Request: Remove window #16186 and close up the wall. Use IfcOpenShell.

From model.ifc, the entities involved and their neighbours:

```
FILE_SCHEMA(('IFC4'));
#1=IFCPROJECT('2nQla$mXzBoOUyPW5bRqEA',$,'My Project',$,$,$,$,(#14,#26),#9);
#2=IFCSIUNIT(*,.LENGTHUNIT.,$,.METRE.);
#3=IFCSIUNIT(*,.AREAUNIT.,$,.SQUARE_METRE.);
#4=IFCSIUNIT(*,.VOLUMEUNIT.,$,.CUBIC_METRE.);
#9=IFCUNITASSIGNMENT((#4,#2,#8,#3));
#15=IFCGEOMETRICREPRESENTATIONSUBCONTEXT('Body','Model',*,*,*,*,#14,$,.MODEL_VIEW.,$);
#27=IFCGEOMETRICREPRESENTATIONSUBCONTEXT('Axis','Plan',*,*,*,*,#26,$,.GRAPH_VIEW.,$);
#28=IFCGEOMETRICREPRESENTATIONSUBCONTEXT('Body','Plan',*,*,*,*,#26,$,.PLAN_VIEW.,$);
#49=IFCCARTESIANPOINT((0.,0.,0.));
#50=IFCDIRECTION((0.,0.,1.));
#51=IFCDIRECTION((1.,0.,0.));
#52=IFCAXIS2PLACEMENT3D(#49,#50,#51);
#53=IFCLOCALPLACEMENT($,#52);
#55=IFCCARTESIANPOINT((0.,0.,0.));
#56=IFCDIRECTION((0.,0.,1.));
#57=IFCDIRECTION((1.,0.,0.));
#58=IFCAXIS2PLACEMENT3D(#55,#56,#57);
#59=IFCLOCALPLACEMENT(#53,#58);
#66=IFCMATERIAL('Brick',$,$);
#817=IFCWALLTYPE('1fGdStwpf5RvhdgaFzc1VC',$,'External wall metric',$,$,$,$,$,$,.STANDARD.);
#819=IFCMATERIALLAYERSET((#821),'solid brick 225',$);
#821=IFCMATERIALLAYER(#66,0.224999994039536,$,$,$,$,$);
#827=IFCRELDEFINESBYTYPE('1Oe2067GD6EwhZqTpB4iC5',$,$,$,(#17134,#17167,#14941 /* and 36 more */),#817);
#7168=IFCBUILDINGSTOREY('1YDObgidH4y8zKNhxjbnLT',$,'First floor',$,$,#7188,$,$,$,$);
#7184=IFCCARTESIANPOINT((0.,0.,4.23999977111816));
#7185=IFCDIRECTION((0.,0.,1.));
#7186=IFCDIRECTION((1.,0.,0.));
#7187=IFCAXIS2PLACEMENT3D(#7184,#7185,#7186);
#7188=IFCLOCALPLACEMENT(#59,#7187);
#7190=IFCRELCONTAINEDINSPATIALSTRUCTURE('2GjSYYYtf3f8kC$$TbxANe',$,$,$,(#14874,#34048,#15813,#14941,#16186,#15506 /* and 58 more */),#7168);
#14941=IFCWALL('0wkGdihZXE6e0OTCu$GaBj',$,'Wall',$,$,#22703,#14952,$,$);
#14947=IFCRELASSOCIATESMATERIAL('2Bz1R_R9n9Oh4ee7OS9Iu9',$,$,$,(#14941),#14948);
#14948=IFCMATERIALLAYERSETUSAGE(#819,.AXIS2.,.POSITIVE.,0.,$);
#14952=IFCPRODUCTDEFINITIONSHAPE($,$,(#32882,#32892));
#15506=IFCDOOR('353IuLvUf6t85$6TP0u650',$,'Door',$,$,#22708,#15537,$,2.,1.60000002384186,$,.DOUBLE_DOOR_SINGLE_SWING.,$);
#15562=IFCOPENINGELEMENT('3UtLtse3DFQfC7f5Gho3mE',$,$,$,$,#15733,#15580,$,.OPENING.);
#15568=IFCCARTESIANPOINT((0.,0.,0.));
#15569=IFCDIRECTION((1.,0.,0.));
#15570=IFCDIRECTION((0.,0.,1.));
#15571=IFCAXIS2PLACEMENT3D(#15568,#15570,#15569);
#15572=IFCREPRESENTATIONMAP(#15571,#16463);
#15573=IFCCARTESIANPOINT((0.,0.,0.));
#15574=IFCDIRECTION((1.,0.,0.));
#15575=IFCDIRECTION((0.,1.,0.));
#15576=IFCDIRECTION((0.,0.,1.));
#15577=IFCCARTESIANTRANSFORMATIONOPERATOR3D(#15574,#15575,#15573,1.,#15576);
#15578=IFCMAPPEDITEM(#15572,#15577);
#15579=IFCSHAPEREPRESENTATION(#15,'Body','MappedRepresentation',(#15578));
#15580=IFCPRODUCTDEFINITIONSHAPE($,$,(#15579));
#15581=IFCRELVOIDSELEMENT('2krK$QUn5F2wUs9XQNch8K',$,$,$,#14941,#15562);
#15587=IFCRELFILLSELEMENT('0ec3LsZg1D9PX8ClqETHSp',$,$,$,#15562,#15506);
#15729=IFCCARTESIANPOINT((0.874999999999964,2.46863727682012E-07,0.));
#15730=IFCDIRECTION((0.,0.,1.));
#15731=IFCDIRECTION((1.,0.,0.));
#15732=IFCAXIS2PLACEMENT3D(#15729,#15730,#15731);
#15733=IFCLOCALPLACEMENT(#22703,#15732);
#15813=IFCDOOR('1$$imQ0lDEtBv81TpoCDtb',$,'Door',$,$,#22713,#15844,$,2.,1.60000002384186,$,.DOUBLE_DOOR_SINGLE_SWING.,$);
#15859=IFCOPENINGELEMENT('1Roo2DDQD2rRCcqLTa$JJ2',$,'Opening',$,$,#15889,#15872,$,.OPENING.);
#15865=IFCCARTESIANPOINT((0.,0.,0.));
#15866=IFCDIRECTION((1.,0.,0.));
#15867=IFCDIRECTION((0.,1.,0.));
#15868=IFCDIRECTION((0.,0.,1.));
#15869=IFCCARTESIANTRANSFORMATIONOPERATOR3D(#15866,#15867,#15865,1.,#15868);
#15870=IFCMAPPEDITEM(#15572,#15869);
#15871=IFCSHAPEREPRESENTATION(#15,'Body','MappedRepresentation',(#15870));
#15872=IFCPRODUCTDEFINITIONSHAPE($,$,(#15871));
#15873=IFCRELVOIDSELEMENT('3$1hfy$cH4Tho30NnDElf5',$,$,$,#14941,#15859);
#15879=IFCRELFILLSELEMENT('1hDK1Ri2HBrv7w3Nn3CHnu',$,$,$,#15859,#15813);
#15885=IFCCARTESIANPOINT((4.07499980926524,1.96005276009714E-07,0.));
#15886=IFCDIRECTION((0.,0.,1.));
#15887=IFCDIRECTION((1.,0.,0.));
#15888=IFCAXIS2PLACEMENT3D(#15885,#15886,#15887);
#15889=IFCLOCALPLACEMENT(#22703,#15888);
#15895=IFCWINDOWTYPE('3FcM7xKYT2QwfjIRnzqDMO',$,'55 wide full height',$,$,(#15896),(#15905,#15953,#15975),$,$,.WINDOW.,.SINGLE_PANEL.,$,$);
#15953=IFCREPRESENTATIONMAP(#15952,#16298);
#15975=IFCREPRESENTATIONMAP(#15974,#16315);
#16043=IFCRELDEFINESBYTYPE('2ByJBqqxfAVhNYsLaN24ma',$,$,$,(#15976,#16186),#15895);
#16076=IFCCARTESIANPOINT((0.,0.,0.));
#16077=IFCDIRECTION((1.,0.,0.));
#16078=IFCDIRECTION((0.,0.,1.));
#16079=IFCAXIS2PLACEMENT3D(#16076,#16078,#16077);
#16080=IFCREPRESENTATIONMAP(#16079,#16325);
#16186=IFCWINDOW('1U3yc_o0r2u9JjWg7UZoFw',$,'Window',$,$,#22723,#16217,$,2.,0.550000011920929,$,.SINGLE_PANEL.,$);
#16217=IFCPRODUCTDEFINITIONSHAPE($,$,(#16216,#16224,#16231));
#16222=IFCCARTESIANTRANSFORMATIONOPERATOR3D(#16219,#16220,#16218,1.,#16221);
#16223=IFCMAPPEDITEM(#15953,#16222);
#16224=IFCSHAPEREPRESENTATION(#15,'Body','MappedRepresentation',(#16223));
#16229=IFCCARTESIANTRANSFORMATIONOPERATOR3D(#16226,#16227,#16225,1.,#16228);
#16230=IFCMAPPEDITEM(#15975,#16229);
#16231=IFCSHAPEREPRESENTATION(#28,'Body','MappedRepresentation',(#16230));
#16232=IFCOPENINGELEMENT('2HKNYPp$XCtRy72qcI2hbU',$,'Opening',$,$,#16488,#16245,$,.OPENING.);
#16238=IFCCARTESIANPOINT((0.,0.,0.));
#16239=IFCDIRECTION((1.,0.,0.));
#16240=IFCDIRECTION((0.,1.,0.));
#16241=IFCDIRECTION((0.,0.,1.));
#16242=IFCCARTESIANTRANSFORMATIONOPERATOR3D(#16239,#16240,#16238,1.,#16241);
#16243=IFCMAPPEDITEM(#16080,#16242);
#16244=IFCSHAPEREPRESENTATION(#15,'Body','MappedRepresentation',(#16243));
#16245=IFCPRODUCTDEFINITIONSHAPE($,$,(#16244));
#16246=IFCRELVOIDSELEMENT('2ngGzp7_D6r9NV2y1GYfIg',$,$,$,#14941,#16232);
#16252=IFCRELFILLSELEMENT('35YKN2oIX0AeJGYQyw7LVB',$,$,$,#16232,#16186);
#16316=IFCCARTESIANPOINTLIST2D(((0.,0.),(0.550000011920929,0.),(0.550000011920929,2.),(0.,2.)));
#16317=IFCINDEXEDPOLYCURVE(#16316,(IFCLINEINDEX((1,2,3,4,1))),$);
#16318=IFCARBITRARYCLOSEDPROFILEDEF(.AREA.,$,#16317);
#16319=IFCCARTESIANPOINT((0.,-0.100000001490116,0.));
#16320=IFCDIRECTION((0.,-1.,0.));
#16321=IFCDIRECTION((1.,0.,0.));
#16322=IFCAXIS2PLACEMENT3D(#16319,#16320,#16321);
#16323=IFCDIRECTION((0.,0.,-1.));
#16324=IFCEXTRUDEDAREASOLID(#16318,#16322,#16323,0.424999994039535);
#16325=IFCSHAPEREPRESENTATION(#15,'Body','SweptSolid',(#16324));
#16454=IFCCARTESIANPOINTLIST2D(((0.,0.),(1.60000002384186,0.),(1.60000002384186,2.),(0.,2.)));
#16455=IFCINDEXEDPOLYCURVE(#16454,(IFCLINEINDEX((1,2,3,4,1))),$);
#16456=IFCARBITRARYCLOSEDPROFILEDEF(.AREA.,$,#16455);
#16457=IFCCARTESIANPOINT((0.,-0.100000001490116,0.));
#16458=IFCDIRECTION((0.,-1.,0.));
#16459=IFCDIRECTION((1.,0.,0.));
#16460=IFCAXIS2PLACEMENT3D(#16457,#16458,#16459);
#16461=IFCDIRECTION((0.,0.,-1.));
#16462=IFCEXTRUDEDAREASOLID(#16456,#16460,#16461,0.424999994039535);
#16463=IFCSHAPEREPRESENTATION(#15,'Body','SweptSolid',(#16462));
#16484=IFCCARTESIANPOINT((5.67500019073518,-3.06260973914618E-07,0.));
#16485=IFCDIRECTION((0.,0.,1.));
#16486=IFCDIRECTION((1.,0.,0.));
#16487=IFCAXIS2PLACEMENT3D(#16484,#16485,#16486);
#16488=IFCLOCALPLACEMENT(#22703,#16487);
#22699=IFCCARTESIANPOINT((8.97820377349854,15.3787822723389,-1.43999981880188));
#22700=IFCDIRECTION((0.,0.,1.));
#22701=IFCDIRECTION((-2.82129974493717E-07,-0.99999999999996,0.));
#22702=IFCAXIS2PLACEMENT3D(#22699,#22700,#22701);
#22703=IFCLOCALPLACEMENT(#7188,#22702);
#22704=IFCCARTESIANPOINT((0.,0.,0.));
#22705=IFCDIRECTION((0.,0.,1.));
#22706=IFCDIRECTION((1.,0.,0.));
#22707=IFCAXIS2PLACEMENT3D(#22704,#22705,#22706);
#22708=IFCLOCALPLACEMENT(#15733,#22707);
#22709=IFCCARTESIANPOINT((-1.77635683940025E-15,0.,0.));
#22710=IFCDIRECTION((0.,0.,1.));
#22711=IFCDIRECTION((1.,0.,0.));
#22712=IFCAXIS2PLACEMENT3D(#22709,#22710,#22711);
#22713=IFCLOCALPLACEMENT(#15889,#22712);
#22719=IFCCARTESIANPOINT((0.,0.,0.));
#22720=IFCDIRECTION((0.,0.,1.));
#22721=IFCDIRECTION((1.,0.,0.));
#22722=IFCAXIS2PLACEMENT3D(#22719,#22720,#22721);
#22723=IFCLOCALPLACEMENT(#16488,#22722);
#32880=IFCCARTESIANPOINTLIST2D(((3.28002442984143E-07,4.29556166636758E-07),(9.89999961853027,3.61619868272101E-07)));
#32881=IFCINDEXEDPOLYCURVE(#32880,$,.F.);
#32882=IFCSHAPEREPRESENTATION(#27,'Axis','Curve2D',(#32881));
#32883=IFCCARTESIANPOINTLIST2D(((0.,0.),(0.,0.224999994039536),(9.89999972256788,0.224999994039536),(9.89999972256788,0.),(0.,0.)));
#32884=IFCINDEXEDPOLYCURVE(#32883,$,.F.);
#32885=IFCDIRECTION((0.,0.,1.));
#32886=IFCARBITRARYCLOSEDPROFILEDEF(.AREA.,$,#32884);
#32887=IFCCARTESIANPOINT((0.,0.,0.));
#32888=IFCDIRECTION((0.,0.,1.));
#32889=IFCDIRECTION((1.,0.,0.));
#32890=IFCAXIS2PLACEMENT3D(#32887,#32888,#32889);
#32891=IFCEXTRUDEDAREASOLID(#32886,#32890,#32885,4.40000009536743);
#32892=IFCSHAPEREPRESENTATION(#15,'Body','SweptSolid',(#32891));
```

```python
import ifcopenshell
import ifcopenshell.api.feature
import ifcopenshell.api.root
import ifcopenshell.geom
import ifcopenshell.util.shape

model = ifcopenshell.open("model.ifc")
settings = ifcopenshell.geom.settings()


def volume(element):
    """Net volume in cubic metres, openings subtracted."""
    shape = ifcopenshell.geom.create_shape(settings, element)
    return ifcopenshell.util.shape.get_volume(shape.geometry)


window = model.by_guid("1U3yc_o0r2u9JjWg7UZoFw")
opening = window.FillsVoids[0].RelatingOpeningElement
wall = opening.VoidsElements[0].RelatingBuildingElement
before = volume(wall)

ifcopenshell.api.root.remove_product(model, product=window)
ifcopenshell.api.feature.remove_feature(model, feature=opening)

after = volume(wall)

print(f"wall volume {before:.3f} -> {after:.3f} m3")

model.write("model_v2.ifc")
```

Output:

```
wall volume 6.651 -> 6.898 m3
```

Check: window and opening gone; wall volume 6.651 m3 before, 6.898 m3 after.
